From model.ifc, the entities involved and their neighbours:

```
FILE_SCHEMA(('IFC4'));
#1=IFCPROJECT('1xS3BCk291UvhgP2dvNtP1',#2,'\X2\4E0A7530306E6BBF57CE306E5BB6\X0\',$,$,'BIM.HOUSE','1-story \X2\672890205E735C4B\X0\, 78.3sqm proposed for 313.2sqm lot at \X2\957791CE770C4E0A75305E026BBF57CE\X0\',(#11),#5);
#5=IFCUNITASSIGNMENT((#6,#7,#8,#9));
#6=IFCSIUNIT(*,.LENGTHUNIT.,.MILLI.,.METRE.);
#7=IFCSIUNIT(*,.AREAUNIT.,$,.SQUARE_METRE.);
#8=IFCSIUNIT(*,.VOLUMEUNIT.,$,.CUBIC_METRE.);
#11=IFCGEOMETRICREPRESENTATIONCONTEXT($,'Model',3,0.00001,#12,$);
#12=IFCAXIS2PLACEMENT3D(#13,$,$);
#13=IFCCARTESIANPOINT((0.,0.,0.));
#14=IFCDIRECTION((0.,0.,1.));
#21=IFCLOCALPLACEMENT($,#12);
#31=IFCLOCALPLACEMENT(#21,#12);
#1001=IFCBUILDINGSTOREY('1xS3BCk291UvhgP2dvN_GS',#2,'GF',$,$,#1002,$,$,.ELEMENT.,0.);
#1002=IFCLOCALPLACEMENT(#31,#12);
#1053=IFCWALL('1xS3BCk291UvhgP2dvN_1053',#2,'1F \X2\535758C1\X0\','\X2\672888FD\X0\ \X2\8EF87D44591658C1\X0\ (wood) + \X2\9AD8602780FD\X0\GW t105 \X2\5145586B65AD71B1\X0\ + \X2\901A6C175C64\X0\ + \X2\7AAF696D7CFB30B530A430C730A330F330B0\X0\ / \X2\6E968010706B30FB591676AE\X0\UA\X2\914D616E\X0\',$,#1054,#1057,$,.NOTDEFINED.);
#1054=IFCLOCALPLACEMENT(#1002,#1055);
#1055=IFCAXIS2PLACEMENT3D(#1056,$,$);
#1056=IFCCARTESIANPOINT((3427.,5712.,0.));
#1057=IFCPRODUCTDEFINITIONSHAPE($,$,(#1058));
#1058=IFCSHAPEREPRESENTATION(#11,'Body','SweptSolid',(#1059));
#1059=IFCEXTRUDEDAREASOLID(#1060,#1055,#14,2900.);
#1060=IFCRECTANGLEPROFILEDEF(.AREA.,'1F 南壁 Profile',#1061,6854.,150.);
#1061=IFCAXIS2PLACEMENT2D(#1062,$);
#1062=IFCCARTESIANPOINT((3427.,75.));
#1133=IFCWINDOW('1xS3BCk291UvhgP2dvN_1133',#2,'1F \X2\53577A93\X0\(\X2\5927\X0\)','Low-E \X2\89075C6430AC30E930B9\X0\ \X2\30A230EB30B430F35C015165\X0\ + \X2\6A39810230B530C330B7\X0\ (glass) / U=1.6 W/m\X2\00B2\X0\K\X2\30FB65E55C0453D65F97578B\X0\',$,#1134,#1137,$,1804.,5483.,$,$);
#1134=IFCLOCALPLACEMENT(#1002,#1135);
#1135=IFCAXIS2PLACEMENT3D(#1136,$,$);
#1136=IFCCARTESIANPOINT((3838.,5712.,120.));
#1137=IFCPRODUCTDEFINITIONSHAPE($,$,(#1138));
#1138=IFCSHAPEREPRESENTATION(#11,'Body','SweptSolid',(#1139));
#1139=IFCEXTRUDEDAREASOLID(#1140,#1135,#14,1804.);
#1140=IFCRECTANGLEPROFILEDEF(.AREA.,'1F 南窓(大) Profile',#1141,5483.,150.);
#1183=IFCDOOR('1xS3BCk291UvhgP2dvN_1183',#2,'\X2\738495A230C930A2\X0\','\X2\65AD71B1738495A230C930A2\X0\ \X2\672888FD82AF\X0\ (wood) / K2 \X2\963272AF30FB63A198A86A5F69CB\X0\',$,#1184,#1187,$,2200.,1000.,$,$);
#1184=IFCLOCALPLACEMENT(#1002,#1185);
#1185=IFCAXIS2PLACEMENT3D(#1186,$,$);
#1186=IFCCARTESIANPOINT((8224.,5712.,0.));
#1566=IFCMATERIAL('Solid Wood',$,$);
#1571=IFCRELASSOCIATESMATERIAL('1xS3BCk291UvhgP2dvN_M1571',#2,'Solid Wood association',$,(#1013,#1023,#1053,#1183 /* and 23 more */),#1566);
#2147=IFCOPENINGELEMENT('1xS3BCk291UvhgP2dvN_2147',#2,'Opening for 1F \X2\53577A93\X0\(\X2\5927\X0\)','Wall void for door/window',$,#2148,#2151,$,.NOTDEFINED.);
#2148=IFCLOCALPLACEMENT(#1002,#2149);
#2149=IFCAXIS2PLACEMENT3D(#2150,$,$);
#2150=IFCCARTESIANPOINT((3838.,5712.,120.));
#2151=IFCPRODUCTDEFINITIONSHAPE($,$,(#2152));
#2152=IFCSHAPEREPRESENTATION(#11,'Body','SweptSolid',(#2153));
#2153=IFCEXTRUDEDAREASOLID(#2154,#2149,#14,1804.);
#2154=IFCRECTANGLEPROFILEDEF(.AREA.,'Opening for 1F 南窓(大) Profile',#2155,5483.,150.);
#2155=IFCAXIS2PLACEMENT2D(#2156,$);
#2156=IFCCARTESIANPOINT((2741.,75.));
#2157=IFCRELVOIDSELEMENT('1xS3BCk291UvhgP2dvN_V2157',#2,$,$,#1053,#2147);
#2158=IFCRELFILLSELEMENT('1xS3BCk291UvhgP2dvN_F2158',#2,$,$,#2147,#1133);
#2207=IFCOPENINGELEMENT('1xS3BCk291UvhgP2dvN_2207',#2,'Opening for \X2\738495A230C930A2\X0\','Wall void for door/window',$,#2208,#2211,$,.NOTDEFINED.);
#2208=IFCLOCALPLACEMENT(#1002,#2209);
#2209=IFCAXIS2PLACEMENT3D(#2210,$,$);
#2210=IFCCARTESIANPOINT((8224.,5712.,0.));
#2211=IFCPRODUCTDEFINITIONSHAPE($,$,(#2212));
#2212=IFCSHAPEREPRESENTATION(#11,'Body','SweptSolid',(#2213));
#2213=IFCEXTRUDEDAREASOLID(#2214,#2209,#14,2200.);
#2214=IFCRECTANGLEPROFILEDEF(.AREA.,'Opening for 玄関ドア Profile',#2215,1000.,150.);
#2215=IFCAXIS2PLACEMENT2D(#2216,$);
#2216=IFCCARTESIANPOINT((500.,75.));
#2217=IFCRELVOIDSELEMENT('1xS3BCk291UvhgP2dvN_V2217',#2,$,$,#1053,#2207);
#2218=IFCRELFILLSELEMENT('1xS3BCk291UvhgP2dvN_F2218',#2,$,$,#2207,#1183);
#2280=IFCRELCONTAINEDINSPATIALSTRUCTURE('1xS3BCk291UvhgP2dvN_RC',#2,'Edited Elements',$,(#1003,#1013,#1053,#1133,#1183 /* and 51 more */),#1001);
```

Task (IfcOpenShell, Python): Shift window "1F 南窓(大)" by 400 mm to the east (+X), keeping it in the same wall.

```python
import ifcopenshell
import ifcopenshell.api.geometry
import ifcopenshell.util.placement

model = ifcopenshell.open("model.ifc")

window = model.by_guid("1xS3BCk291UvhgP2dvN_1133")
opening = window.FillsVoids[0].RelatingOpeningElement
wall = opening.VoidsElements[0].RelatingBuildingElement

wall_matrix = ifcopenshell.util.placement.get_local_placement(wall.ObjectPlacement)
shift = wall_matrix[:3, 0] * 400.0
before = ifcopenshell.util.placement.get_local_placement(window.ObjectPlacement)[:3, 3].copy()

# The window is not placed relative to its opening, so move both.
for product in (opening, window):
    matrix = ifcopenshell.util.placement.get_local_placement(product.ObjectPlacement)
    matrix[:3, 3] += shift
    ifcopenshell.api.geometry.edit_object_placement(model, product=product, matrix=matrix, is_si=False)

after = ifcopenshell.util.placement.get_local_placement(window.ObjectPlacement)[:3, 3]
print("window moved by", (after - before).round(3) + 0.0)

model.write("model_v2.ifc")
```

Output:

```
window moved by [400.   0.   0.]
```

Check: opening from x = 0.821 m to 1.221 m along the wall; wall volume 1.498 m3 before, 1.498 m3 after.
